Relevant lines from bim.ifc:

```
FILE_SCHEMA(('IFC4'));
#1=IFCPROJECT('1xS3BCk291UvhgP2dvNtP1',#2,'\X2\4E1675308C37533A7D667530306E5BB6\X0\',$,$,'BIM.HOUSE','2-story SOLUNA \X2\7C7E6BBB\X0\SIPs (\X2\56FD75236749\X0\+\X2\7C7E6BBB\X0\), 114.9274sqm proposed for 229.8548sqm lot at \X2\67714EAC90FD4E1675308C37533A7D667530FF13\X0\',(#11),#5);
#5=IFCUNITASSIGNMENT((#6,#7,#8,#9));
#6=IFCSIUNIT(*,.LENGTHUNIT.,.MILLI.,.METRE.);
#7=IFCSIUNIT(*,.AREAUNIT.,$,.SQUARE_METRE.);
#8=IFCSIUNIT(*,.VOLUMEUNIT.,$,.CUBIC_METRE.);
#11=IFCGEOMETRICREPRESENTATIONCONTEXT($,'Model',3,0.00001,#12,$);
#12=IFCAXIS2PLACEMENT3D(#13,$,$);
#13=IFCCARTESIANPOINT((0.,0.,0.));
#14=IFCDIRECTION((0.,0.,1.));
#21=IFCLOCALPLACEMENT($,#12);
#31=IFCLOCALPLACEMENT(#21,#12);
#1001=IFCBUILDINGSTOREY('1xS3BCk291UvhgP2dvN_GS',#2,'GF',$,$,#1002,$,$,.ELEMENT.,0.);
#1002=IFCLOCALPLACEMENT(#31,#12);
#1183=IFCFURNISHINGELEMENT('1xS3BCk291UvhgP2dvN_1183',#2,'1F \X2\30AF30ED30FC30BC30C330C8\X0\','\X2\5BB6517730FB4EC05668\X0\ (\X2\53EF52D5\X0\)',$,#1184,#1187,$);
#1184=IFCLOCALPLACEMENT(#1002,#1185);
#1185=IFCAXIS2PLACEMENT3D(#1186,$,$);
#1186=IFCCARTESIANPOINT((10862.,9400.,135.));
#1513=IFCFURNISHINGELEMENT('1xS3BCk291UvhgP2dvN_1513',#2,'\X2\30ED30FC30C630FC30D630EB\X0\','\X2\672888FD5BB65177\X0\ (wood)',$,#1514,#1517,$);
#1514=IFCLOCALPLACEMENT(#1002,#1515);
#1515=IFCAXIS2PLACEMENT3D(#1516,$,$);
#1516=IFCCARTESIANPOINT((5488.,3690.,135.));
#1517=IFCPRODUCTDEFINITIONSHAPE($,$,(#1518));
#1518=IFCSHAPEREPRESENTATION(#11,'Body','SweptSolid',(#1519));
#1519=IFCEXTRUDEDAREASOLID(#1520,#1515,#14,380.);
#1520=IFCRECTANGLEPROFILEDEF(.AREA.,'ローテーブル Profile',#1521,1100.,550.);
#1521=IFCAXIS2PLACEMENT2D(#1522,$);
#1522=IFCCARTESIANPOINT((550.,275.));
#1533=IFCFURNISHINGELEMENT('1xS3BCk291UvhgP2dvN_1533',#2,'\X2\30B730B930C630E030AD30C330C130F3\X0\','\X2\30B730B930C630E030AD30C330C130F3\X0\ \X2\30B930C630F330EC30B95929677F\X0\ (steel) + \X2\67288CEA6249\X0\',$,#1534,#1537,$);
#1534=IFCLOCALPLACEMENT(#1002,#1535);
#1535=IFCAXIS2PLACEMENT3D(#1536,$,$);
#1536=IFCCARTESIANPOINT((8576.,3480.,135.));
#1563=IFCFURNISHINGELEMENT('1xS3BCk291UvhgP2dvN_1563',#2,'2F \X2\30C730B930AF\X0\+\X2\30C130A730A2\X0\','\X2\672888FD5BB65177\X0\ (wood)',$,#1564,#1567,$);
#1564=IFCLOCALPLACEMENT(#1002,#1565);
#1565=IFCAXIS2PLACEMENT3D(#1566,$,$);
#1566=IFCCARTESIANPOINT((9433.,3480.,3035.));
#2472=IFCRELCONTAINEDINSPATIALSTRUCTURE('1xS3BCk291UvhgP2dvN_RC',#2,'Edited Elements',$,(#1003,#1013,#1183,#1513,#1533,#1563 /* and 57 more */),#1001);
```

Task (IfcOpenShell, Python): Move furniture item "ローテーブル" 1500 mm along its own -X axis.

```python
import ifcopenshell
import ifcopenshell.api.geometry
import ifcopenshell.util.placement

model = ifcopenshell.open("bim.ifc")

item = model.by_id(1513)
matrix = ifcopenshell.util.placement.get_local_placement(item.ObjectPlacement)
matrix[:3, 3] -= matrix[:3, 0] * 1500.0
ifcopenshell.api.geometry.edit_object_placement(model, product=item, matrix=matrix, is_si=False)

print(ifcopenshell.util.placement.get_local_placement(item.ObjectPlacement).round(3) + 0.0)

model.write("bim_rev.ifc")
```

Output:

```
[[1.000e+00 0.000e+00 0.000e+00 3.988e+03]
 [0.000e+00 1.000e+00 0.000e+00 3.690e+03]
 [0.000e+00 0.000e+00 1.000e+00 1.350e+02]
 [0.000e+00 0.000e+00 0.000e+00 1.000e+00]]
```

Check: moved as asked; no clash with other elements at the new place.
